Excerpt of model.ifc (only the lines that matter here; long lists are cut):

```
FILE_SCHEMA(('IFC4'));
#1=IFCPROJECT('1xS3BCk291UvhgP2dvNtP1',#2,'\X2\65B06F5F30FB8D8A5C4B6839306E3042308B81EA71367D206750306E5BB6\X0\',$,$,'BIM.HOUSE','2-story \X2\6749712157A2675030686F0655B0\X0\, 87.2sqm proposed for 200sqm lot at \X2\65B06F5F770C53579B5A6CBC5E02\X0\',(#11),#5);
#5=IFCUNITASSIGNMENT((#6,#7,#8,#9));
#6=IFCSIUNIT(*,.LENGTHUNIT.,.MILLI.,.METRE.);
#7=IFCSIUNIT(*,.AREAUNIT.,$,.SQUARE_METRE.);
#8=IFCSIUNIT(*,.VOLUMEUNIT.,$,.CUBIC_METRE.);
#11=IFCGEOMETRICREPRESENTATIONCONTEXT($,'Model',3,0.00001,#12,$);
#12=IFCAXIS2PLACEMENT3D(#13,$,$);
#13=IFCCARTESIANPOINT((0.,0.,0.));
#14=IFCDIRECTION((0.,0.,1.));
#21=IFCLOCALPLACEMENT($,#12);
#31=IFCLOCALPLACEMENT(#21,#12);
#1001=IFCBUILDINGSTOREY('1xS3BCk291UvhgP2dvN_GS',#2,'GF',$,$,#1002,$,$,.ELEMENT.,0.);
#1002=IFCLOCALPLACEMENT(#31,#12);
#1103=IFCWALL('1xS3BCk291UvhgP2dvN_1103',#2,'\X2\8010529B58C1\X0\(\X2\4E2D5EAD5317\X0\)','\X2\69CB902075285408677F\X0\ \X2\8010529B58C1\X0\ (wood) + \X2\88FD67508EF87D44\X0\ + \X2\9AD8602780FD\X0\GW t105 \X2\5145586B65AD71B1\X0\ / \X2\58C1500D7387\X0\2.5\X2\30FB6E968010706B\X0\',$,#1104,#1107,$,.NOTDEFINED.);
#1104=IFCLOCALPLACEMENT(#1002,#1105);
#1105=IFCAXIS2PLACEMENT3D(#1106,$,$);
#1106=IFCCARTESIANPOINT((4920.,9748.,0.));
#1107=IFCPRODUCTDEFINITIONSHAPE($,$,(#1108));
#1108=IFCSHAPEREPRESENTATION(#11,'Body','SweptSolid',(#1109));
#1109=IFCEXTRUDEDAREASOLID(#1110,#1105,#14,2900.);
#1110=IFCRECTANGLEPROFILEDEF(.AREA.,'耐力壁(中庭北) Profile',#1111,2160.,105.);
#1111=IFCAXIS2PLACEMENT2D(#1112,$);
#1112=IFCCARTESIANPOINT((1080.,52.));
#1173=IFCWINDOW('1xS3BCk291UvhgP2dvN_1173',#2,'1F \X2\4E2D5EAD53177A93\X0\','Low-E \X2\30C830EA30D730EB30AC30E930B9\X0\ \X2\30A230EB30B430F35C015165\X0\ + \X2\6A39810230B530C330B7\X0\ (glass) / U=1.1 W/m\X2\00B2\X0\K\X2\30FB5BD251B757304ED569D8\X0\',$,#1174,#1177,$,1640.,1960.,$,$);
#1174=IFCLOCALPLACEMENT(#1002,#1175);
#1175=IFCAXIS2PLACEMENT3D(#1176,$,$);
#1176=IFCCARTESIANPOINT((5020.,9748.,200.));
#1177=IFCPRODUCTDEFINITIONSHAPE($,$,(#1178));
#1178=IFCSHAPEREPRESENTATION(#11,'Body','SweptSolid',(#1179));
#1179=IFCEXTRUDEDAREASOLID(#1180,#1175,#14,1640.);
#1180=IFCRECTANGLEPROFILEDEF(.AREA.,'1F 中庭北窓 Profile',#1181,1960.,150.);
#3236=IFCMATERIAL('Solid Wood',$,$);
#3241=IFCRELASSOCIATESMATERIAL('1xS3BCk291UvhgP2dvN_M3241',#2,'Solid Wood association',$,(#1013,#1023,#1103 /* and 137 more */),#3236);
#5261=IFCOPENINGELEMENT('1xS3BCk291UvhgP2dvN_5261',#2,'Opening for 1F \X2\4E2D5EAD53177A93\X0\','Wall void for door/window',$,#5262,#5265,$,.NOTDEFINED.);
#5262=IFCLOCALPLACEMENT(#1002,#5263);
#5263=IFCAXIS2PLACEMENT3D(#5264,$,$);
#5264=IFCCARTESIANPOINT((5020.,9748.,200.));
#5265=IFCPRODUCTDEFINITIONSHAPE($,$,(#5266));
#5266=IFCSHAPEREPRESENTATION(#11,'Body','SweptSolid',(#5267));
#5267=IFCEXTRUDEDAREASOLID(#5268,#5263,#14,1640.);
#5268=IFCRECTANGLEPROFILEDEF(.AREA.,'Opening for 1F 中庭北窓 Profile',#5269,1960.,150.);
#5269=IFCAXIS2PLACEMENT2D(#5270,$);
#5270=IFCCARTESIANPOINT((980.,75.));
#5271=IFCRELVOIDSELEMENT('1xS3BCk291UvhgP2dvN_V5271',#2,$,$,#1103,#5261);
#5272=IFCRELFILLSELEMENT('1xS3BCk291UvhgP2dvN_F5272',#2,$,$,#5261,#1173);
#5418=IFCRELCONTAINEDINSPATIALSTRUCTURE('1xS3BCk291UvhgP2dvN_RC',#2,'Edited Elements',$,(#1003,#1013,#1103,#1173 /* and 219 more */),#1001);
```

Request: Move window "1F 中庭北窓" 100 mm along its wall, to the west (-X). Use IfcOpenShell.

```python
import ifcopenshell
import ifcopenshell.api.geometry
import ifcopenshell.util.placement

model = ifcopenshell.open("model.ifc")

window = model.by_guid("1xS3BCk291UvhgP2dvN_1173")
opening = window.FillsVoids[0].RelatingOpeningElement
wall = opening.VoidsElements[0].RelatingBuildingElement

wall_matrix = ifcopenshell.util.placement.get_local_placement(wall.ObjectPlacement)
shift = wall_matrix[:3, 0] * -100.0
before = ifcopenshell.util.placement.get_local_placement(window.ObjectPlacement)[:3, 3].copy()

# The window is not placed relative to its opening, so move both.
for product in (opening, window):
    matrix = ifcopenshell.util.placement.get_local_placement(product.ObjectPlacement)
    matrix[:3, 3] += shift
    ifcopenshell.api.geometry.edit_object_placement(model, product=product, matrix=matrix, is_si=False)

after = ifcopenshell.util.placement.get_local_placement(window.ObjectPlacement)[:3, 3]
print("window moved by", (after - before).round(3) + 0.0)

model.write("model_rev.ifc")
```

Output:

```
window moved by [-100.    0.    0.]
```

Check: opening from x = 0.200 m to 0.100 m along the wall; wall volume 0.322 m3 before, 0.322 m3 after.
